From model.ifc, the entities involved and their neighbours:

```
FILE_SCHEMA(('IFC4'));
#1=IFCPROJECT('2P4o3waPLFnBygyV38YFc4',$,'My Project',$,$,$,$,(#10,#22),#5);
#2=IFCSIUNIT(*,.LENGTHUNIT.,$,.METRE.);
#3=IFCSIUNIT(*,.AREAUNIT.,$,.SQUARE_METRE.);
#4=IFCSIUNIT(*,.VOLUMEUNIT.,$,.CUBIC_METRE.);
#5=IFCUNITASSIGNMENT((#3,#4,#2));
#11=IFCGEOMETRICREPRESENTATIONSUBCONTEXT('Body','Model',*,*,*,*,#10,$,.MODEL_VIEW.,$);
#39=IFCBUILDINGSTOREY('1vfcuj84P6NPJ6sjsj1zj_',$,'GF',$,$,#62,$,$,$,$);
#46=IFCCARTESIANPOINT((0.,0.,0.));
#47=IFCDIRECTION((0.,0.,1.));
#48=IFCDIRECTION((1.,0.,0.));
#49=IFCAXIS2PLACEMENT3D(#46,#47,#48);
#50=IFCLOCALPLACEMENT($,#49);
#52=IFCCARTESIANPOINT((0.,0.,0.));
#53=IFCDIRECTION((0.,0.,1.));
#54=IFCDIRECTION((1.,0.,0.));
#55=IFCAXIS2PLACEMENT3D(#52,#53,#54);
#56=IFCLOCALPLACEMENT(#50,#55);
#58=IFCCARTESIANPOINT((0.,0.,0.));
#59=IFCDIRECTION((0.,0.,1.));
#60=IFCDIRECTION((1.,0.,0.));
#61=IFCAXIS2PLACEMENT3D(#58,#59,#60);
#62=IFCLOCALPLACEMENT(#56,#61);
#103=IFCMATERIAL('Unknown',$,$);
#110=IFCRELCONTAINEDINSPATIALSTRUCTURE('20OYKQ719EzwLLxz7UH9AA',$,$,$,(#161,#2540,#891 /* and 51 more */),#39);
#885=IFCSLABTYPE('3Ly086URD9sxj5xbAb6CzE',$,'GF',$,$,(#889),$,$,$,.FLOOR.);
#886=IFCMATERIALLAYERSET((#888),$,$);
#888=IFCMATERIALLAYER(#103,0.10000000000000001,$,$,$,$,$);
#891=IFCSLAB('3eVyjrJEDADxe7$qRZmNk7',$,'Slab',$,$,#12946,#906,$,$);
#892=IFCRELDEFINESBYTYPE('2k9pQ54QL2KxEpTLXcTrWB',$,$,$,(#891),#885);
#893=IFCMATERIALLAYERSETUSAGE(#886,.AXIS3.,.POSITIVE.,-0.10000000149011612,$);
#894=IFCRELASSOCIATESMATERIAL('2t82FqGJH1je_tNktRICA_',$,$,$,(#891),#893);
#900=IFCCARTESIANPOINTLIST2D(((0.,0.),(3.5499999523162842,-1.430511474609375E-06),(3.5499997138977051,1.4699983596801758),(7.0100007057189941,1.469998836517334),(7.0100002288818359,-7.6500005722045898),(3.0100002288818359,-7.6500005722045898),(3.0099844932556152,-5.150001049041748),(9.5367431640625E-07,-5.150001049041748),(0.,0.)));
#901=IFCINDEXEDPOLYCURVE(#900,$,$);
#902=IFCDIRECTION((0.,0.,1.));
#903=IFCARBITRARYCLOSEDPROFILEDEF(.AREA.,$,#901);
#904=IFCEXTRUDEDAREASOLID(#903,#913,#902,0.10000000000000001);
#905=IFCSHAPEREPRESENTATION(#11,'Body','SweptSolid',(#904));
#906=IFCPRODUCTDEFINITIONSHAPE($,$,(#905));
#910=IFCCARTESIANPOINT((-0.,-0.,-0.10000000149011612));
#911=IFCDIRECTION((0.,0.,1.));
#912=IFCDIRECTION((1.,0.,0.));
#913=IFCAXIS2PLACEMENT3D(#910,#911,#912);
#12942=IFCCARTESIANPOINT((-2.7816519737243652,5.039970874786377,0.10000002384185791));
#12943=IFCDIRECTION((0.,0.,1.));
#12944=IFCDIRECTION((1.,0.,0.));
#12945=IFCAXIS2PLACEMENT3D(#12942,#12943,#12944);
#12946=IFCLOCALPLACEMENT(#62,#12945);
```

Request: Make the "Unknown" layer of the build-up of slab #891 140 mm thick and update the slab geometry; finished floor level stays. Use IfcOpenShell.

```python
import ifcopenshell
import ifcopenshell.util.element
import ifcopenshell.util.representation
import ifcopenshell.util.unit

model = ifcopenshell.open("model.ifc")
unit_scale = ifcopenshell.util.unit.calculate_unit_scale(model)

layer_set = model.by_id(886)
layer = next(l for l in layer_set.MaterialLayers if l.Material and l.Material.Name == "Unknown")
change = 0.14 / unit_scale - layer.LayerThickness
layer.LayerThickness += change

# Geometry does not follow the layer set by itself.
slabs = [e for e in ifcopenshell.util.element.get_elements_by_material(model, layer_set) if e.is_a("IfcSlab")]
for slab in sorted(slabs, key=lambda e: e.id()):
    body = ifcopenshell.util.representation.get_representation(slab, "Model", "Body")
    solid = body.Items[0]
    old_depth = solid.Depth
    solid.Depth += change
    # Extruded upwards: lower the start of the extrusion so the top stays.
    x, y, z = solid.Position.Location.Coordinates
    solid.Position.Location = model.createIfcCartesianPoint((x, y, z - change))
    print(slab.id(), f"{old_depth:g} -> {solid.Depth:g}")

# The layers are counted up from the underside, which has moved.
for usage in {ifcopenshell.util.element.get_material(slab) for slab in slabs}:
    usage.OffsetFromReferenceLine -= change

model.write("model_updated.ifc")
```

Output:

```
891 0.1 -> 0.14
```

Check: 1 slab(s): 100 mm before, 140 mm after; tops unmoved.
